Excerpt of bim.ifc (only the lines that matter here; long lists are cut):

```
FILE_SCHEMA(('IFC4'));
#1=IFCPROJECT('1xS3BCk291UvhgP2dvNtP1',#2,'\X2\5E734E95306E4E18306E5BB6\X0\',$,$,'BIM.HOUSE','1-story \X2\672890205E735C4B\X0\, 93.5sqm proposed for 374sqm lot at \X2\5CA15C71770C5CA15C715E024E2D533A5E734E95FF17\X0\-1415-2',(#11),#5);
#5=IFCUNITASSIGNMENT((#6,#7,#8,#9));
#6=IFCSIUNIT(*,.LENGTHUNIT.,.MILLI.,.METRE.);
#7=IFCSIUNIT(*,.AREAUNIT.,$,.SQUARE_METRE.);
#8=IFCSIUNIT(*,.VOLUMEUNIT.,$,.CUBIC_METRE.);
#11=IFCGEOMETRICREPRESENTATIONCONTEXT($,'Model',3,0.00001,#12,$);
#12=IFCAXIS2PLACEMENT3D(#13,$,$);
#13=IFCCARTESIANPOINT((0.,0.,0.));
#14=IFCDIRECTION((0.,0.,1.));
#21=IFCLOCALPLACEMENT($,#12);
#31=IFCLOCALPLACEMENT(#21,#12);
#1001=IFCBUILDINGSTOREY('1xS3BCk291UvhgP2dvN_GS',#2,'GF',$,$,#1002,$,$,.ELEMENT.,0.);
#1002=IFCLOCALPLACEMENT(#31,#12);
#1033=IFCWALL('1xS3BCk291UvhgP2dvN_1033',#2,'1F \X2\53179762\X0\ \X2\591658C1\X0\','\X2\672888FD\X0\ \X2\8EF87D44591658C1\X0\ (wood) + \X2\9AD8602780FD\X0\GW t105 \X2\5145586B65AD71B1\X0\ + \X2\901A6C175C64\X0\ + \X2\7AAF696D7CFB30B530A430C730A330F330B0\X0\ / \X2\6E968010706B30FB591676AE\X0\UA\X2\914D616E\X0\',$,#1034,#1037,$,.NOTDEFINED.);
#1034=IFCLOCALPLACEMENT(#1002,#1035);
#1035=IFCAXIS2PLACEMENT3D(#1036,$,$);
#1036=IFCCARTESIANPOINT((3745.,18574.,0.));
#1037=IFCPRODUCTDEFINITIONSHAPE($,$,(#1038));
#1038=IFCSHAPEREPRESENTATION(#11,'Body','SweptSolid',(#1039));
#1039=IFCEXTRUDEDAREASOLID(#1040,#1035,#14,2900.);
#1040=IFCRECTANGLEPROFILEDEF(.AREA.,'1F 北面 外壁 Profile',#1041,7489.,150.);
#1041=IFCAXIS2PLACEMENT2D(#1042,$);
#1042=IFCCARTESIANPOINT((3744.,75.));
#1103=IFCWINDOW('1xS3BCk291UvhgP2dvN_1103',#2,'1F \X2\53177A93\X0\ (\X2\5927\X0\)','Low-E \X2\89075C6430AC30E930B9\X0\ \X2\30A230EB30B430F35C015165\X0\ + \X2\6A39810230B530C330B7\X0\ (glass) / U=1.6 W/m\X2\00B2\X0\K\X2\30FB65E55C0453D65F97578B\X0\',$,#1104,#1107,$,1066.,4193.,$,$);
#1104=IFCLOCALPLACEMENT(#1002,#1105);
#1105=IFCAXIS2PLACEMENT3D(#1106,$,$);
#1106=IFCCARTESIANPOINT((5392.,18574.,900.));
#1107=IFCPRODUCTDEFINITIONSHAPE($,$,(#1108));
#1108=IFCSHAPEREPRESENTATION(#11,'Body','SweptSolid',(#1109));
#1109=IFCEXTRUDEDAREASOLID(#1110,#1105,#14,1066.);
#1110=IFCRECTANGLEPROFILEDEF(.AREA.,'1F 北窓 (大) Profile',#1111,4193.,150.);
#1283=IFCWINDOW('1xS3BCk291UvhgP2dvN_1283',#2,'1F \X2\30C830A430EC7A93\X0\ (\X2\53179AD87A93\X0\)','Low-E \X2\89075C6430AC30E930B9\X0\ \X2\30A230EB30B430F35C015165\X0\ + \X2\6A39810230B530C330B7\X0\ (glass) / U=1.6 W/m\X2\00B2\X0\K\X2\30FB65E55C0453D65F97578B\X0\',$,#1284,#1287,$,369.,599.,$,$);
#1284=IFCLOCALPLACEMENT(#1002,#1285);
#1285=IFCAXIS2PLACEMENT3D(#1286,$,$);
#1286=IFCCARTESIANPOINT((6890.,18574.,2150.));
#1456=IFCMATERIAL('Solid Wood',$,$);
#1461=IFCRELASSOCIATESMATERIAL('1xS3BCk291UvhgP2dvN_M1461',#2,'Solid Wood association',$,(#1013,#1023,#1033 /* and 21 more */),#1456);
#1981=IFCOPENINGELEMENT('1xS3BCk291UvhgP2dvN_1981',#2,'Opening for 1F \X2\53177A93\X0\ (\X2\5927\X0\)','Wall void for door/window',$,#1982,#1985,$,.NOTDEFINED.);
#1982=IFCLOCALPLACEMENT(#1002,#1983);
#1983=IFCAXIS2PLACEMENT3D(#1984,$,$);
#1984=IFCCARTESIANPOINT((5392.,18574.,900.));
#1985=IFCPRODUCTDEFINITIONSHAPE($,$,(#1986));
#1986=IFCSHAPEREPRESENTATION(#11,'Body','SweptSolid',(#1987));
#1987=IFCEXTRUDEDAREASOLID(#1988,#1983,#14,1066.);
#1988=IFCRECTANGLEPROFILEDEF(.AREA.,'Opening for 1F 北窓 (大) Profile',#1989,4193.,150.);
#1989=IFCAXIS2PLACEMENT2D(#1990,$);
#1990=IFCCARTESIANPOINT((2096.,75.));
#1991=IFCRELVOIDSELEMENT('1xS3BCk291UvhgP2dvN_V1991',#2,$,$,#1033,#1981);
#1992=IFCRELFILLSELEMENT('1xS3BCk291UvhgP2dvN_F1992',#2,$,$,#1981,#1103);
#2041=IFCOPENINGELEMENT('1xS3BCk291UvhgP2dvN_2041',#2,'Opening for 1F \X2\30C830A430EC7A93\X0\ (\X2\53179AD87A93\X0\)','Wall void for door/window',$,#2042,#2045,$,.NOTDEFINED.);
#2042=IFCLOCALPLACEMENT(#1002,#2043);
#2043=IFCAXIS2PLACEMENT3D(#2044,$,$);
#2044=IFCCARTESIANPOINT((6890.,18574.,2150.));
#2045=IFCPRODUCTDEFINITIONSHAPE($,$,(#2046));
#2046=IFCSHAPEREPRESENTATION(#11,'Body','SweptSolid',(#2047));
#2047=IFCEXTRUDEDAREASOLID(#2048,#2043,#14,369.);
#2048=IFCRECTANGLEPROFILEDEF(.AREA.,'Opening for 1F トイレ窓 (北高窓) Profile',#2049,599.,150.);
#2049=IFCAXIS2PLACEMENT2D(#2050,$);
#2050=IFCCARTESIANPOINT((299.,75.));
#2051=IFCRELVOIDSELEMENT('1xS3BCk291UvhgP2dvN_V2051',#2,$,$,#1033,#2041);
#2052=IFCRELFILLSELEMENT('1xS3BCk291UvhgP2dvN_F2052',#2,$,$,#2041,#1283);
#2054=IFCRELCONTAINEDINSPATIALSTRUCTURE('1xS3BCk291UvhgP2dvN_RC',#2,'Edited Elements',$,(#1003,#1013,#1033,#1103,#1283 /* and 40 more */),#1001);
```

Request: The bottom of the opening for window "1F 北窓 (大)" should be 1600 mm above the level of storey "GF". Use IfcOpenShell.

```python
import numpy as np
import ifcopenshell
import ifcopenshell.api.geometry
import ifcopenshell.geom
import ifcopenshell.util.element
import ifcopenshell.util.placement
import ifcopenshell.util.shape
import ifcopenshell.util.unit

model = ifcopenshell.open("bim.ifc")
unit_scale = ifcopenshell.util.unit.calculate_unit_scale(model)

window = model.by_guid("1xS3BCk291UvhgP2dvN_1103")
opening = window.FillsVoids[0].RelatingOpeningElement
storey = ifcopenshell.util.element.get_container(window, ifc_class="IfcBuildingStorey")
level = ifcopenshell.util.placement.get_local_placement(storey.ObjectPlacement)[2, 3]

# The opening's origin need not be at the sill, so measure its lowest point.
shape = ifcopenshell.geom.create_shape(ifcopenshell.geom.settings(), opening)
bottom = ifcopenshell.util.shape.get_shape_bottom_elevation(shape, shape.geometry) / unit_scale
dz = level + 1.6 / unit_scale - bottom

shift = np.array([0.0, 0.0, dz])
# The window is not placed relative to its opening, so move both.
for product in (opening, window):
    matrix = ifcopenshell.util.placement.get_local_placement(product.ObjectPlacement)
    matrix[:3, 3] += shift
    ifcopenshell.api.geometry.edit_object_placement(model, product=product, matrix=matrix, is_si=False)

print(f"moved by {dz * unit_scale:+.3f} m")

model.write("bim_updated.ifc")
```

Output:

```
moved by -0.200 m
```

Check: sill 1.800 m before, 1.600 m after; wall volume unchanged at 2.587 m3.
